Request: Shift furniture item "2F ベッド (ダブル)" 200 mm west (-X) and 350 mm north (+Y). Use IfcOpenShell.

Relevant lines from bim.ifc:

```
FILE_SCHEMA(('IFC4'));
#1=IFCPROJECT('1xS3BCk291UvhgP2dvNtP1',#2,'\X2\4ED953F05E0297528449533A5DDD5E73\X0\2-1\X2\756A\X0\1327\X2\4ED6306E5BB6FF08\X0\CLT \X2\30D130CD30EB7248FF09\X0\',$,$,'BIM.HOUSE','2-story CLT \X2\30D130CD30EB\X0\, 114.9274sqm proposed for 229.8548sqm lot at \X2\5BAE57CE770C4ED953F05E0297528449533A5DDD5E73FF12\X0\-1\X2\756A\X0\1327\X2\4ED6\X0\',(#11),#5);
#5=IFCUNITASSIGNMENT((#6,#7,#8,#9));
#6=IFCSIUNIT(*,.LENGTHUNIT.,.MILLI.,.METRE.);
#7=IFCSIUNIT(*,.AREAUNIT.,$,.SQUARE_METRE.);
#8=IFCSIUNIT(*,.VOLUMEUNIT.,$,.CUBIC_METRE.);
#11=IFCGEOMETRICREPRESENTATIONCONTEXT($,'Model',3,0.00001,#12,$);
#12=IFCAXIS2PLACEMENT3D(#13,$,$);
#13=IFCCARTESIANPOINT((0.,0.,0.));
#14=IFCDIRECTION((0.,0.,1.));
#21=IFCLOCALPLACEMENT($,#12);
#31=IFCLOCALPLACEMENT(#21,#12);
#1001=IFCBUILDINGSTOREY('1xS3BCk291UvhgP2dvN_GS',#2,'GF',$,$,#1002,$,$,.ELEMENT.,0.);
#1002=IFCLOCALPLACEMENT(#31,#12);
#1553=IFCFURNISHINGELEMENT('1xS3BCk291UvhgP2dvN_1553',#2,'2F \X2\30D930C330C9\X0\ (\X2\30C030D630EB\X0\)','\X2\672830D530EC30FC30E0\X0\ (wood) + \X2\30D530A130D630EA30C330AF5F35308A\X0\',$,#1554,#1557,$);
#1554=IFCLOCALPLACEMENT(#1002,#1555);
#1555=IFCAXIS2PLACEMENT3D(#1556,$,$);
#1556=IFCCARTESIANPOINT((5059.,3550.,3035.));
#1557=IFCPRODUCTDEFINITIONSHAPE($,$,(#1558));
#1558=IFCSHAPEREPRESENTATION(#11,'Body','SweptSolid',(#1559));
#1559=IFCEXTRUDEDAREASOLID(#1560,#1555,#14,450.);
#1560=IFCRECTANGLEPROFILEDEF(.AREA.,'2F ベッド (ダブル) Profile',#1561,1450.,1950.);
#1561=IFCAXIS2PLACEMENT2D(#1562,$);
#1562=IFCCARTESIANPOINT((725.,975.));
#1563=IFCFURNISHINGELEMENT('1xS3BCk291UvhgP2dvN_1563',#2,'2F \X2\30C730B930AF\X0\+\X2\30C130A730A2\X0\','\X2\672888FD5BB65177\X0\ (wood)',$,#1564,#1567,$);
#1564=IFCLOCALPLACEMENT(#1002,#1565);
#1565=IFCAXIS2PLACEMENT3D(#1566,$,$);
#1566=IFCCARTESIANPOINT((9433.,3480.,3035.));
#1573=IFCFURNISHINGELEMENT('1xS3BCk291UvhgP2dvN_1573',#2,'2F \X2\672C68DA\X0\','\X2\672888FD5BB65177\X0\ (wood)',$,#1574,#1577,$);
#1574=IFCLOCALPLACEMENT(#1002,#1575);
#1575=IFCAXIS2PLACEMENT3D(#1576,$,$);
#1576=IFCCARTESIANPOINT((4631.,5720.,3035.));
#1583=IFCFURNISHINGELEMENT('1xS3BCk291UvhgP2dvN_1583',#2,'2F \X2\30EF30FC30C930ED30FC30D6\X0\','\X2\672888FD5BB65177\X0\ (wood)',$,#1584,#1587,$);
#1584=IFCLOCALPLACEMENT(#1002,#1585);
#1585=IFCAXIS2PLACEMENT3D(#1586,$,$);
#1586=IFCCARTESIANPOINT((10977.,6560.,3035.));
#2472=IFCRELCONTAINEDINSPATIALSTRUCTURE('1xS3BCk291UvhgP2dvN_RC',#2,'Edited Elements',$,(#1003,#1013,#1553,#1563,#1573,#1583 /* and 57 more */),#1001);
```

```python
import ifcopenshell
import ifcopenshell.api.geometry
import ifcopenshell.util.placement

model = ifcopenshell.open("bim.ifc")

item = model.by_id(1553)
matrix = ifcopenshell.util.placement.get_local_placement(item.ObjectPlacement)
matrix[0, 3] -= 200.0
matrix[1, 3] += 350.0
ifcopenshell.api.geometry.edit_object_placement(model, product=item, matrix=matrix, is_si=False)

print(ifcopenshell.util.placement.get_local_placement(item.ObjectPlacement).round(3) + 0.0)

model.write("bim_edited.ifc")
```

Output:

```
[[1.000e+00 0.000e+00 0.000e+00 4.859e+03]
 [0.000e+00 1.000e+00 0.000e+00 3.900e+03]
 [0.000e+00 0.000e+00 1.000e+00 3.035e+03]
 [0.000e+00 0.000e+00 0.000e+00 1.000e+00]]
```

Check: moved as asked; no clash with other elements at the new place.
